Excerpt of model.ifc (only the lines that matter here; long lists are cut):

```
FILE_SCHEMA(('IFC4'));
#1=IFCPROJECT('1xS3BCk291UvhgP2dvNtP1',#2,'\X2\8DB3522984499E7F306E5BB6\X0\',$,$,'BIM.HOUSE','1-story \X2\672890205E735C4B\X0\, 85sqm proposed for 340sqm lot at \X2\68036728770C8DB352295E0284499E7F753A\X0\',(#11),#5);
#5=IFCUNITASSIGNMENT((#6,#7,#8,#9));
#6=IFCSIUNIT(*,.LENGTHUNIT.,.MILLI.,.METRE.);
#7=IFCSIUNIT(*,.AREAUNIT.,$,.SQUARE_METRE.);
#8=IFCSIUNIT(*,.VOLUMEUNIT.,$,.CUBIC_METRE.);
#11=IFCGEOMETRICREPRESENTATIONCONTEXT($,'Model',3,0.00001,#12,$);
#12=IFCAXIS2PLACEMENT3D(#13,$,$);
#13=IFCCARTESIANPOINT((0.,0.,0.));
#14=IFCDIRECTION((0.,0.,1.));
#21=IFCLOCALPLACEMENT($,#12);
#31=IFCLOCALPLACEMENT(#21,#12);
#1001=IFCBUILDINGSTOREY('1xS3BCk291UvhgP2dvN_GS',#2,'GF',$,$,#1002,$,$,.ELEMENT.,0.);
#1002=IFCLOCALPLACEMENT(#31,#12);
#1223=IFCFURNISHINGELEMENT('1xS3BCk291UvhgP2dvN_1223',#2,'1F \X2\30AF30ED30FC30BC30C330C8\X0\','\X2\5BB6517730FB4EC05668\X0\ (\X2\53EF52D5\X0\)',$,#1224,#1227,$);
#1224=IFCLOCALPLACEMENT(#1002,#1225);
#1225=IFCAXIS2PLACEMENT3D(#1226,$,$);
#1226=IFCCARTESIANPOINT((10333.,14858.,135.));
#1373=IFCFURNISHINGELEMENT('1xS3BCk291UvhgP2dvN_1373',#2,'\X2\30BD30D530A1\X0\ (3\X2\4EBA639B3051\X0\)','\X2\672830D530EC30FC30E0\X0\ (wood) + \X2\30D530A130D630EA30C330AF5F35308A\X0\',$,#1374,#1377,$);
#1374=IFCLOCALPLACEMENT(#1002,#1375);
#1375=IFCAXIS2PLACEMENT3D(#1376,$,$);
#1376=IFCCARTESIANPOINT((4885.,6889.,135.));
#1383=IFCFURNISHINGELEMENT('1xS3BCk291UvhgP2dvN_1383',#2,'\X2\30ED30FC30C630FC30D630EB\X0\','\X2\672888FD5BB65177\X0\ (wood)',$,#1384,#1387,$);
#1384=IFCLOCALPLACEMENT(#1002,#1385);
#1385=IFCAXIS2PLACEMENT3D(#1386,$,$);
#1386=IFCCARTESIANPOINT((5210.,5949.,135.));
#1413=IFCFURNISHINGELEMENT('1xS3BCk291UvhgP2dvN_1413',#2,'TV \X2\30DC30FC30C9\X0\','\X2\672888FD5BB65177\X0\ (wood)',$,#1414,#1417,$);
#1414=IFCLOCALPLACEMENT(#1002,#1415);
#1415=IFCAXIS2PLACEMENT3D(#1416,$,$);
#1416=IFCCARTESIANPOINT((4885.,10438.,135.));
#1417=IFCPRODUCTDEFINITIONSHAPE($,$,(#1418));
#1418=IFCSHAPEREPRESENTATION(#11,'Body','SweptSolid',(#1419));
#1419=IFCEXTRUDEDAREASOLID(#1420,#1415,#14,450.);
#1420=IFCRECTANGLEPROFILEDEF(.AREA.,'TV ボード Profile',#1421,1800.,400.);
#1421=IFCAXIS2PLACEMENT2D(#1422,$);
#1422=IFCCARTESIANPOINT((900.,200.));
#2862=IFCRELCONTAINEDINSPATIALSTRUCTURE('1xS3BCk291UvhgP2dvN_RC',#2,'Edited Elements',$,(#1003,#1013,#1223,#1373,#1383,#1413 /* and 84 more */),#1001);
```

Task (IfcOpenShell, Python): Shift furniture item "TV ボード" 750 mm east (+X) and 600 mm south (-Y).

```python
import ifcopenshell
import ifcopenshell.api.geometry
import ifcopenshell.util.placement

model = ifcopenshell.open("model.ifc")

item = model.by_id(1413)
matrix = ifcopenshell.util.placement.get_local_placement(item.ObjectPlacement)
matrix[0, 3] += 750.0
matrix[1, 3] -= 600.0
ifcopenshell.api.geometry.edit_object_placement(model, product=item, matrix=matrix, is_si=False)

print(ifcopenshell.util.placement.get_local_placement(item.ObjectPlacement).round(3) + 0.0)

model.write("model_v2.ifc")
```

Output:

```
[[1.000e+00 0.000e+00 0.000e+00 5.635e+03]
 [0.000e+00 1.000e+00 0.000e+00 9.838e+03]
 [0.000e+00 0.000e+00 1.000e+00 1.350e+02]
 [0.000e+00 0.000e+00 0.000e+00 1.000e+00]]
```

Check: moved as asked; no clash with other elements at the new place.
